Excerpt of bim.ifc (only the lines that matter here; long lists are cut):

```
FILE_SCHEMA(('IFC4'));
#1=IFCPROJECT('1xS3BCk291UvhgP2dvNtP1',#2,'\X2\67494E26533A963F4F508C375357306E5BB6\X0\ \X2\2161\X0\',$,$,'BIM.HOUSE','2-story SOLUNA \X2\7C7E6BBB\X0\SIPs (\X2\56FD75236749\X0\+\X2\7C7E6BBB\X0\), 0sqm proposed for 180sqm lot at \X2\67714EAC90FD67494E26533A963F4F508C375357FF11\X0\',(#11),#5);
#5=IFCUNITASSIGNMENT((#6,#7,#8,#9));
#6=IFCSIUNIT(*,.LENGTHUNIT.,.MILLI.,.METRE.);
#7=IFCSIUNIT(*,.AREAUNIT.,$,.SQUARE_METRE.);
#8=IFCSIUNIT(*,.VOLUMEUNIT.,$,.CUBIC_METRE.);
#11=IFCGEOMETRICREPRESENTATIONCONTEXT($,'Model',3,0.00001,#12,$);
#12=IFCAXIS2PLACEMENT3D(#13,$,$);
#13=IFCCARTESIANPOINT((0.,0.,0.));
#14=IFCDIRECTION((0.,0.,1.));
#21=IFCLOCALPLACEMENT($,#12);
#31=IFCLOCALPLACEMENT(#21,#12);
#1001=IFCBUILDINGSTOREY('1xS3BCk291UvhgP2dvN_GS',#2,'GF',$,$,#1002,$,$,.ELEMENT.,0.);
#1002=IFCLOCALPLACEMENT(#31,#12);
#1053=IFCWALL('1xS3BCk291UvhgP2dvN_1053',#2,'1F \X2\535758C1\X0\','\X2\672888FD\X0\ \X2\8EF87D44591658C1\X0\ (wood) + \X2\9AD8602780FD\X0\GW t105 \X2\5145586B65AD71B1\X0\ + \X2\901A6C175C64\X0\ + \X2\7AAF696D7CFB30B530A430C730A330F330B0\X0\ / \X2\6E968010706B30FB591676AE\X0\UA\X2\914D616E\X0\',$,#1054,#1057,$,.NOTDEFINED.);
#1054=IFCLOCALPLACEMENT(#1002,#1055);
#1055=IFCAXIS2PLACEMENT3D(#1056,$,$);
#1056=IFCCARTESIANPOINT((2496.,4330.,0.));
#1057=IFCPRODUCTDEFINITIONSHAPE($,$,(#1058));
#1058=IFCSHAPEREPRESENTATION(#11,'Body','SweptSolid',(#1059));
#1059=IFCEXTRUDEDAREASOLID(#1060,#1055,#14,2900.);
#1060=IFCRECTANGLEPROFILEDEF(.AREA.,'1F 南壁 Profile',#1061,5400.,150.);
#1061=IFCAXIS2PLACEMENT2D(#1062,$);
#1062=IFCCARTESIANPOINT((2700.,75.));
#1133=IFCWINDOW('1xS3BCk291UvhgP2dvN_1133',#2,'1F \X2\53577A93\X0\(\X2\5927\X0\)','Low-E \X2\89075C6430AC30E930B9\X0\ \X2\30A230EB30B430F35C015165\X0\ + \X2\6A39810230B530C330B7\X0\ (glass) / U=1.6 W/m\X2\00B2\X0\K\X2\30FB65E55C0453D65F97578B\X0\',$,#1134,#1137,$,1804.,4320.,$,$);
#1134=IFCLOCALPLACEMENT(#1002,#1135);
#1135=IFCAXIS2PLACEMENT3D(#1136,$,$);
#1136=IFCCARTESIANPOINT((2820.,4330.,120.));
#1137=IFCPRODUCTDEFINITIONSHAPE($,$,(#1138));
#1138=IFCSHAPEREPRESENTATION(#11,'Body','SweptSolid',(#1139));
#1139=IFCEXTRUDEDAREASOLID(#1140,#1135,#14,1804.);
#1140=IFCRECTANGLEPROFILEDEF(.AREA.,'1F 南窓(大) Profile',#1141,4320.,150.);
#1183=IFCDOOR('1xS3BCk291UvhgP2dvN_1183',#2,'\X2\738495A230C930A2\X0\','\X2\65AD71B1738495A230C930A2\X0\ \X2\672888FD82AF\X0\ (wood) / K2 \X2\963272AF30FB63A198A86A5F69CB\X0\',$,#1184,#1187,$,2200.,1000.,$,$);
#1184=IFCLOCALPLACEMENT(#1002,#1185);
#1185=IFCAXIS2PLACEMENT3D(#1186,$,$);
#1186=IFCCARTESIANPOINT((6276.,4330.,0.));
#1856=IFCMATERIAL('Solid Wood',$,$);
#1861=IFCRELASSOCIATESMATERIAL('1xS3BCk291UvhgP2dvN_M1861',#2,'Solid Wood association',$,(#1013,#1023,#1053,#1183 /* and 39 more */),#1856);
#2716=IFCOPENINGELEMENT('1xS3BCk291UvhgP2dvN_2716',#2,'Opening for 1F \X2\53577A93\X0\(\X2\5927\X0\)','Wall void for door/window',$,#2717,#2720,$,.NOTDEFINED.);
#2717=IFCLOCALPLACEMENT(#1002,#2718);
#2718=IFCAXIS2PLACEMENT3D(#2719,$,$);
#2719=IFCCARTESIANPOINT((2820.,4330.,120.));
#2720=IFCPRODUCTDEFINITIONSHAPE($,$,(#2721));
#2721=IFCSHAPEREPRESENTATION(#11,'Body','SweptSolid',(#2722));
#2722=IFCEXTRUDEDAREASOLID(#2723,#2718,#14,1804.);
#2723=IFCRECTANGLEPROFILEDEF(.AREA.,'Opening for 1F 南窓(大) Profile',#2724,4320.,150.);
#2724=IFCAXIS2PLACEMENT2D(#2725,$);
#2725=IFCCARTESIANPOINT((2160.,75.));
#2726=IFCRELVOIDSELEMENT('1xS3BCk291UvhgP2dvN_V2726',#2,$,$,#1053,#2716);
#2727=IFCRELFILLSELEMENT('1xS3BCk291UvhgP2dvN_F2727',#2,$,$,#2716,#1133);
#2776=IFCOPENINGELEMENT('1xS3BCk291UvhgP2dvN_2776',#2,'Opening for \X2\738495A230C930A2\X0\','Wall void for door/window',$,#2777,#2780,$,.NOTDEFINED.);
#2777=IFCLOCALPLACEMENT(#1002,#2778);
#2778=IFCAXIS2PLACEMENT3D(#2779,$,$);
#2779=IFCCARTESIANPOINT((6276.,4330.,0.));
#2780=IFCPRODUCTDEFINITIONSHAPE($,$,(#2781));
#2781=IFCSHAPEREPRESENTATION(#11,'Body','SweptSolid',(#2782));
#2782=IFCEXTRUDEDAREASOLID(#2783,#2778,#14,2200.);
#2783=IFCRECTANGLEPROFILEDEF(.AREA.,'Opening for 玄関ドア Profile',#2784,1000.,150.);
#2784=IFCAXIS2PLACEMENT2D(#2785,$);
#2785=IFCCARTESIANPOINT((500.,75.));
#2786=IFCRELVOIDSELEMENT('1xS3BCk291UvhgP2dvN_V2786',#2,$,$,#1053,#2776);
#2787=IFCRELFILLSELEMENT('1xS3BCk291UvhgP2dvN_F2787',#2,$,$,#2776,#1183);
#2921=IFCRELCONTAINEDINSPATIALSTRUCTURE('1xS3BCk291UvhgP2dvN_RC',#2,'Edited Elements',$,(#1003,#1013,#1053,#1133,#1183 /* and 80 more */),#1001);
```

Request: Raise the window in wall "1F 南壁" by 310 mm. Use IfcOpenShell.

```python
import numpy as np
import ifcopenshell
import ifcopenshell.api.geometry
import ifcopenshell.util.placement
import ifcopenshell.util.unit

model = ifcopenshell.open("bim.ifc")
unit_scale = ifcopenshell.util.unit.calculate_unit_scale(model)

window = model.by_guid("1xS3BCk291UvhgP2dvN_1133")
opening = window.FillsVoids[0].RelatingOpeningElement
dz = 310.0

shift = np.array([0.0, 0.0, dz])
# The window is not placed relative to its opening, so move both.
for product in (opening, window):
    matrix = ifcopenshell.util.placement.get_local_placement(product.ObjectPlacement)
    matrix[:3, 3] += shift
    ifcopenshell.api.geometry.edit_object_placement(model, product=product, matrix=matrix, is_si=False)

print(f"moved by {dz * unit_scale:+.3f} m")

model.write("bim_rev.ifc")
```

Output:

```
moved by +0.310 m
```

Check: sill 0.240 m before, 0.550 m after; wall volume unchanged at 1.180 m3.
